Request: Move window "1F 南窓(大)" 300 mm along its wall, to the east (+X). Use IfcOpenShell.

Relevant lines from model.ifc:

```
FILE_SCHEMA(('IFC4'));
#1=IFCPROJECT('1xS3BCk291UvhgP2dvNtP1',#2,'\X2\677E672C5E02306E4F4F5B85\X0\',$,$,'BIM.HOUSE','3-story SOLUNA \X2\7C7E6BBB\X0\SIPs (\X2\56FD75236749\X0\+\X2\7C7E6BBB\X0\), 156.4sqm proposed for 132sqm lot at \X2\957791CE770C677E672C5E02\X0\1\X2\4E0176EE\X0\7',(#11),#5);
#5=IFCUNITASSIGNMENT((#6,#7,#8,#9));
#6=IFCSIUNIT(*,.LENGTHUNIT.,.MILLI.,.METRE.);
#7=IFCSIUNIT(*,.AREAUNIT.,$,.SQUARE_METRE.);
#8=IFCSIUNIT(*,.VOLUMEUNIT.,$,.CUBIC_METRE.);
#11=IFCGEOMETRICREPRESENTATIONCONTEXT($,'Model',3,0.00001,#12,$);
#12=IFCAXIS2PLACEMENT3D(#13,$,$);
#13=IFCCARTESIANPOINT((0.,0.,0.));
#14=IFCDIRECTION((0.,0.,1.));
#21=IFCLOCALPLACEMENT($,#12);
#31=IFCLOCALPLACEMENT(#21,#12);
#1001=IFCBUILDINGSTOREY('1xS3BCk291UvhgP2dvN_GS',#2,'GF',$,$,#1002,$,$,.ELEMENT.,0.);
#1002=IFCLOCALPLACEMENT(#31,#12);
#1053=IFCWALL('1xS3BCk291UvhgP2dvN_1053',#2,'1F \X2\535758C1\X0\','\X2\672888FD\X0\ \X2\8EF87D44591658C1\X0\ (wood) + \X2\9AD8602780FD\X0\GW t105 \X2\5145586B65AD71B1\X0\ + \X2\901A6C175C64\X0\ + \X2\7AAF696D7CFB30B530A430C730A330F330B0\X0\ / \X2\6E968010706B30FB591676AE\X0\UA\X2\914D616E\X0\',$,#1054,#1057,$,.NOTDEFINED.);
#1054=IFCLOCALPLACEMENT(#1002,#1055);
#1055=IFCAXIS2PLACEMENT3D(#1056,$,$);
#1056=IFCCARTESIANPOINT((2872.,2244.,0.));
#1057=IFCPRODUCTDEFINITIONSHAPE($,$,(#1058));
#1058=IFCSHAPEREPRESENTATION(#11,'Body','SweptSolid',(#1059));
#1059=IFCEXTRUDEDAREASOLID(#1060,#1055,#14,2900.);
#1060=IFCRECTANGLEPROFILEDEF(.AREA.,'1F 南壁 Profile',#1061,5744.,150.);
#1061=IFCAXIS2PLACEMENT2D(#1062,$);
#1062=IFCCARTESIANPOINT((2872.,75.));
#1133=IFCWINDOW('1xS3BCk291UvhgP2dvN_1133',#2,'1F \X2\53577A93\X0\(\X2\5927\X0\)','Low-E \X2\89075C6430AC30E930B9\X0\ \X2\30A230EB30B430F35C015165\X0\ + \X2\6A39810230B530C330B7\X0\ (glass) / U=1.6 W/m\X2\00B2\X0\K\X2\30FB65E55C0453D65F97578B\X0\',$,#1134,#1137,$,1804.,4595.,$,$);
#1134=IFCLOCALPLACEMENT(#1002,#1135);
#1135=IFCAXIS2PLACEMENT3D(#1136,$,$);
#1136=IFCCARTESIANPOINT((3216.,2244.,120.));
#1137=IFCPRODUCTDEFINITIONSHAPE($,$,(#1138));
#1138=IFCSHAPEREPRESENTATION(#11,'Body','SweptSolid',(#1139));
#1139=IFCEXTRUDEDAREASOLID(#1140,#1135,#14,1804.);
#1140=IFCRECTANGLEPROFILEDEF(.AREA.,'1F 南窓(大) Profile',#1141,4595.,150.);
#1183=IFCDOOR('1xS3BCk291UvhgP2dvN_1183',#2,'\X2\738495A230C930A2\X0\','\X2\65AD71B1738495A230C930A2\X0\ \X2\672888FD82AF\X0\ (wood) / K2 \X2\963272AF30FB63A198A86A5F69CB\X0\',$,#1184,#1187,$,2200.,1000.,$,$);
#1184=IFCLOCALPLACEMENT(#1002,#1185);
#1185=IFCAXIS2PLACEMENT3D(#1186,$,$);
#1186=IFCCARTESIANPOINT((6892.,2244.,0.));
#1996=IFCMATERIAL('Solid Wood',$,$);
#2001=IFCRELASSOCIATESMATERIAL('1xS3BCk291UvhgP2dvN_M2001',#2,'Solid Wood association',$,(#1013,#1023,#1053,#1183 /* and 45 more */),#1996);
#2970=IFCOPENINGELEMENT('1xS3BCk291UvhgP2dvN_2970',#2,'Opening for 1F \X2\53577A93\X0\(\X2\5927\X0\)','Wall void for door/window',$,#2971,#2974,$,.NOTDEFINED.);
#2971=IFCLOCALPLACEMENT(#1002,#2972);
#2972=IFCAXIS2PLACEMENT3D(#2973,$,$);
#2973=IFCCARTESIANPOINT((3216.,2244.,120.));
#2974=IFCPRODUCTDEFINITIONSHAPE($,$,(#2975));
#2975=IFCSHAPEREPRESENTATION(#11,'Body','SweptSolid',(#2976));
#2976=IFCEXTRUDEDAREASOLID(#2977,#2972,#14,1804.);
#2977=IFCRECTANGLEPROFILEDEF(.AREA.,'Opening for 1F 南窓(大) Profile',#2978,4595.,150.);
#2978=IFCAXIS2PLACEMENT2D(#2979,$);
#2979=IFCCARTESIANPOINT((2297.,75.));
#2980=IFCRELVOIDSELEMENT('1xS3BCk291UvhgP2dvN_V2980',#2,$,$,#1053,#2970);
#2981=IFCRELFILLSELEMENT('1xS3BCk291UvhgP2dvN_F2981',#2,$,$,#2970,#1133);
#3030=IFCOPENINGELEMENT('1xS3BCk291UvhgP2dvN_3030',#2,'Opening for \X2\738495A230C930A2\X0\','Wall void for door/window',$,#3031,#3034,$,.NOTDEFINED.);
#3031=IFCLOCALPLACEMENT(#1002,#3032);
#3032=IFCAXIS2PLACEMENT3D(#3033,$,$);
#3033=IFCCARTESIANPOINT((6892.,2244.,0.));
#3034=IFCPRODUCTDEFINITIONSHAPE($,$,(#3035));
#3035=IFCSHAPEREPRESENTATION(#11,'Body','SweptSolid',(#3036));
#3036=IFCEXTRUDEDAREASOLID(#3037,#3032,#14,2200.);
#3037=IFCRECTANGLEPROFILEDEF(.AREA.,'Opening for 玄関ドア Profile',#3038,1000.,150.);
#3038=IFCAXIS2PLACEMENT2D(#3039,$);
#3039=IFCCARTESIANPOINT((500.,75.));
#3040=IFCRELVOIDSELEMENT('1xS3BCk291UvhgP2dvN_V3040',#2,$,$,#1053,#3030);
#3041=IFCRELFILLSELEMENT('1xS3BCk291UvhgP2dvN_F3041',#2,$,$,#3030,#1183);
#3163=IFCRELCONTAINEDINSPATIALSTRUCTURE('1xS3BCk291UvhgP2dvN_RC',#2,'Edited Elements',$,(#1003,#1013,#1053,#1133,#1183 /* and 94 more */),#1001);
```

```python
import ifcopenshell
import ifcopenshell.api.geometry
import ifcopenshell.util.placement
import ifcopenshell.util.unit

model = ifcopenshell.open("model.ifc")
unit_scale = ifcopenshell.util.unit.calculate_unit_scale(model)

window = model.by_guid("1xS3BCk291UvhgP2dvN_1133")
opening = window.FillsVoids[0].RelatingOpeningElement
wall = opening.VoidsElements[0].RelatingBuildingElement

wall_matrix = ifcopenshell.util.placement.get_local_placement(wall.ObjectPlacement)
shift = wall_matrix[:3, 0] * 0.3 / unit_scale
before = ifcopenshell.util.placement.get_local_placement(window.ObjectPlacement)[:3, 3].copy()

# The window is not placed relative to its opening, so move both.
for product in (opening, window):
    matrix = ifcopenshell.util.placement.get_local_placement(product.ObjectPlacement)
    matrix[:3, 3] += shift
    ifcopenshell.api.geometry.edit_object_placement(model, product=product, matrix=matrix, is_si=False)

after = ifcopenshell.util.placement.get_local_placement(window.ObjectPlacement)[:3, 3]
print("window moved by", (after - before).round(3) + 0.0)

model.write("model_rev.ifc")
```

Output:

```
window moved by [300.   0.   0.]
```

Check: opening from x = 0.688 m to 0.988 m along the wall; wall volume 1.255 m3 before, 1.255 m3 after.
